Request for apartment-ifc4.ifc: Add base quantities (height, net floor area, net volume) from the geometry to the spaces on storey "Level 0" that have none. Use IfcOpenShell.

First a look at what the model holds.

```python
import ifcopenshell
import ifcopenshell.util.element
import ifcopenshell.util.unit

model = ifcopenshell.open("apartment-ifc4.ifc")
print(model.schema)
for unit_type in ("LENGTHUNIT", "AREAUNIT", "VOLUMEUNIT"):
    print(unit_type, ifcopenshell.util.unit.calculate_unit_scale(model, unit_type))
storey = next(s for s in model.by_type("IfcBuildingStorey") if s.Name == "Level 0")
spaces = [e for e in ifcopenshell.util.element.get_decomposition(storey) if e.is_a("IfcSpace")]
for e in sorted(spaces, key=lambda e: e.id()):
    print(e.id(), e.is_a(), e.Name, list(ifcopenshell.util.element.get_psets(e, qtos_only=True)), sep=" | ")
```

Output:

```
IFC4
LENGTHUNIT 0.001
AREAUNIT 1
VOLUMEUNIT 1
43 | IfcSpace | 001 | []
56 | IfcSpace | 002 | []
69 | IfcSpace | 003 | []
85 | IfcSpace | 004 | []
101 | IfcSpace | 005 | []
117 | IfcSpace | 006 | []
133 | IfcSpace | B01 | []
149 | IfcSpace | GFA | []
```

```python
import ifcopenshell
import ifcopenshell.api.pset
import ifcopenshell.geom
import ifcopenshell.util.element
import ifcopenshell.util.shape
import ifcopenshell.util.unit

model = ifcopenshell.open("apartment-ifc4.ifc")
unit_scale = ifcopenshell.util.unit.calculate_unit_scale(model)
area_scale = ifcopenshell.util.unit.calculate_unit_scale(model, "AREAUNIT")
volume_scale = ifcopenshell.util.unit.calculate_unit_scale(model, "VOLUMEUNIT")
settings = ifcopenshell.geom.settings()

storey = next(s for s in model.by_type("IfcBuildingStorey") if s.Name == "Level 0")
spaces = [e for e in ifcopenshell.util.element.get_decomposition(storey) if e.is_a("IfcSpace")]

for e in sorted(spaces, key=lambda e: e.id()):
    if ifcopenshell.util.element.get_psets(e, qtos_only=True, should_inherit=False):
        continue
    # Geometry comes back in metres, in the element's own axes.
    shape = ifcopenshell.geom.create_shape(settings, e)
    values = {
        "Height": ifcopenshell.util.shape.get_z(shape.geometry) / unit_scale,
        "NetFloorArea": ifcopenshell.util.shape.get_footprint_area(shape.geometry) / area_scale,
        "NetVolume": ifcopenshell.util.shape.get_volume(shape.geometry) / volume_scale,
    }
    qto = ifcopenshell.api.pset.add_qto(model, product=e, name="Qto_SpaceBaseQuantities")
    ifcopenshell.api.pset.edit_qto(model, qto=qto, properties=values)
    print(e.id(), {k: round(v, 3) for k, v in values.items()})

model.write("apartment-ifc4_rev.ifc")
```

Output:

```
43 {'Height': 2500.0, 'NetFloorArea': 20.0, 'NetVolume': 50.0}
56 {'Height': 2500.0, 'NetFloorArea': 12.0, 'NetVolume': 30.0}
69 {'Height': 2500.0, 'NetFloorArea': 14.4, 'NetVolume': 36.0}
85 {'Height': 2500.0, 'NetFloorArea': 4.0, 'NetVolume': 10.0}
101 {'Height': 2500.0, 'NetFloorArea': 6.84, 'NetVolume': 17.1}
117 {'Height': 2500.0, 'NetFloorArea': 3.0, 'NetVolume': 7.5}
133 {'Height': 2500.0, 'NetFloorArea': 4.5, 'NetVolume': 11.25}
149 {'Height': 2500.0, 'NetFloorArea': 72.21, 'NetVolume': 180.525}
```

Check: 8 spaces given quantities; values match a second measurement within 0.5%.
